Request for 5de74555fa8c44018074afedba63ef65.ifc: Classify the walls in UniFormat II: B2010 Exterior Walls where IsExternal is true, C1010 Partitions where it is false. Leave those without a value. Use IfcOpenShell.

First a look at what the model holds.

```python
import ifcopenshell
import ifcopenshell.util.element

model = ifcopenshell.open("5de74555fa8c44018074afedba63ef65.ifc")
print(model.schema)
print("classifications:", [c.Name for c in model.by_type("IfcClassification")])
values = [ifcopenshell.util.element.get_pset(e, "Pset_WallCommon", "IsExternal") for e in model.by_type("IfcWall")]
for value in (True, False, None):
    print("IsExternal", value, values.count(value))
```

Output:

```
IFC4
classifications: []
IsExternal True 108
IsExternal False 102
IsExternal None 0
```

```python
import ifcopenshell
import ifcopenshell.api.classification
import ifcopenshell.util.element

model = ifcopenshell.open("5de74555fa8c44018074afedba63ef65.ifc")

system = ifcopenshell.api.classification.add_classification(model, classification="UniFormat II")

walls = model.by_type("IfcWall")
external = {e: ifcopenshell.util.element.get_pset(e, "Pset_WallCommon", "IsExternal") for e in walls}
for flag, code, name in ((True, "B2010", "Exterior Walls"), (False, "C1010", "Partitions")):
    products = [e for e in walls if external[e] is flag]
    ifcopenshell.api.classification.add_reference(
        model, products=products, classification=system, identification=code, name=name
    )
    print(code, len(products))

model.write("5de74555fa8c44018074afedba63ef65_v2.ifc")
```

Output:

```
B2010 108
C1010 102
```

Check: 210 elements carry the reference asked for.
